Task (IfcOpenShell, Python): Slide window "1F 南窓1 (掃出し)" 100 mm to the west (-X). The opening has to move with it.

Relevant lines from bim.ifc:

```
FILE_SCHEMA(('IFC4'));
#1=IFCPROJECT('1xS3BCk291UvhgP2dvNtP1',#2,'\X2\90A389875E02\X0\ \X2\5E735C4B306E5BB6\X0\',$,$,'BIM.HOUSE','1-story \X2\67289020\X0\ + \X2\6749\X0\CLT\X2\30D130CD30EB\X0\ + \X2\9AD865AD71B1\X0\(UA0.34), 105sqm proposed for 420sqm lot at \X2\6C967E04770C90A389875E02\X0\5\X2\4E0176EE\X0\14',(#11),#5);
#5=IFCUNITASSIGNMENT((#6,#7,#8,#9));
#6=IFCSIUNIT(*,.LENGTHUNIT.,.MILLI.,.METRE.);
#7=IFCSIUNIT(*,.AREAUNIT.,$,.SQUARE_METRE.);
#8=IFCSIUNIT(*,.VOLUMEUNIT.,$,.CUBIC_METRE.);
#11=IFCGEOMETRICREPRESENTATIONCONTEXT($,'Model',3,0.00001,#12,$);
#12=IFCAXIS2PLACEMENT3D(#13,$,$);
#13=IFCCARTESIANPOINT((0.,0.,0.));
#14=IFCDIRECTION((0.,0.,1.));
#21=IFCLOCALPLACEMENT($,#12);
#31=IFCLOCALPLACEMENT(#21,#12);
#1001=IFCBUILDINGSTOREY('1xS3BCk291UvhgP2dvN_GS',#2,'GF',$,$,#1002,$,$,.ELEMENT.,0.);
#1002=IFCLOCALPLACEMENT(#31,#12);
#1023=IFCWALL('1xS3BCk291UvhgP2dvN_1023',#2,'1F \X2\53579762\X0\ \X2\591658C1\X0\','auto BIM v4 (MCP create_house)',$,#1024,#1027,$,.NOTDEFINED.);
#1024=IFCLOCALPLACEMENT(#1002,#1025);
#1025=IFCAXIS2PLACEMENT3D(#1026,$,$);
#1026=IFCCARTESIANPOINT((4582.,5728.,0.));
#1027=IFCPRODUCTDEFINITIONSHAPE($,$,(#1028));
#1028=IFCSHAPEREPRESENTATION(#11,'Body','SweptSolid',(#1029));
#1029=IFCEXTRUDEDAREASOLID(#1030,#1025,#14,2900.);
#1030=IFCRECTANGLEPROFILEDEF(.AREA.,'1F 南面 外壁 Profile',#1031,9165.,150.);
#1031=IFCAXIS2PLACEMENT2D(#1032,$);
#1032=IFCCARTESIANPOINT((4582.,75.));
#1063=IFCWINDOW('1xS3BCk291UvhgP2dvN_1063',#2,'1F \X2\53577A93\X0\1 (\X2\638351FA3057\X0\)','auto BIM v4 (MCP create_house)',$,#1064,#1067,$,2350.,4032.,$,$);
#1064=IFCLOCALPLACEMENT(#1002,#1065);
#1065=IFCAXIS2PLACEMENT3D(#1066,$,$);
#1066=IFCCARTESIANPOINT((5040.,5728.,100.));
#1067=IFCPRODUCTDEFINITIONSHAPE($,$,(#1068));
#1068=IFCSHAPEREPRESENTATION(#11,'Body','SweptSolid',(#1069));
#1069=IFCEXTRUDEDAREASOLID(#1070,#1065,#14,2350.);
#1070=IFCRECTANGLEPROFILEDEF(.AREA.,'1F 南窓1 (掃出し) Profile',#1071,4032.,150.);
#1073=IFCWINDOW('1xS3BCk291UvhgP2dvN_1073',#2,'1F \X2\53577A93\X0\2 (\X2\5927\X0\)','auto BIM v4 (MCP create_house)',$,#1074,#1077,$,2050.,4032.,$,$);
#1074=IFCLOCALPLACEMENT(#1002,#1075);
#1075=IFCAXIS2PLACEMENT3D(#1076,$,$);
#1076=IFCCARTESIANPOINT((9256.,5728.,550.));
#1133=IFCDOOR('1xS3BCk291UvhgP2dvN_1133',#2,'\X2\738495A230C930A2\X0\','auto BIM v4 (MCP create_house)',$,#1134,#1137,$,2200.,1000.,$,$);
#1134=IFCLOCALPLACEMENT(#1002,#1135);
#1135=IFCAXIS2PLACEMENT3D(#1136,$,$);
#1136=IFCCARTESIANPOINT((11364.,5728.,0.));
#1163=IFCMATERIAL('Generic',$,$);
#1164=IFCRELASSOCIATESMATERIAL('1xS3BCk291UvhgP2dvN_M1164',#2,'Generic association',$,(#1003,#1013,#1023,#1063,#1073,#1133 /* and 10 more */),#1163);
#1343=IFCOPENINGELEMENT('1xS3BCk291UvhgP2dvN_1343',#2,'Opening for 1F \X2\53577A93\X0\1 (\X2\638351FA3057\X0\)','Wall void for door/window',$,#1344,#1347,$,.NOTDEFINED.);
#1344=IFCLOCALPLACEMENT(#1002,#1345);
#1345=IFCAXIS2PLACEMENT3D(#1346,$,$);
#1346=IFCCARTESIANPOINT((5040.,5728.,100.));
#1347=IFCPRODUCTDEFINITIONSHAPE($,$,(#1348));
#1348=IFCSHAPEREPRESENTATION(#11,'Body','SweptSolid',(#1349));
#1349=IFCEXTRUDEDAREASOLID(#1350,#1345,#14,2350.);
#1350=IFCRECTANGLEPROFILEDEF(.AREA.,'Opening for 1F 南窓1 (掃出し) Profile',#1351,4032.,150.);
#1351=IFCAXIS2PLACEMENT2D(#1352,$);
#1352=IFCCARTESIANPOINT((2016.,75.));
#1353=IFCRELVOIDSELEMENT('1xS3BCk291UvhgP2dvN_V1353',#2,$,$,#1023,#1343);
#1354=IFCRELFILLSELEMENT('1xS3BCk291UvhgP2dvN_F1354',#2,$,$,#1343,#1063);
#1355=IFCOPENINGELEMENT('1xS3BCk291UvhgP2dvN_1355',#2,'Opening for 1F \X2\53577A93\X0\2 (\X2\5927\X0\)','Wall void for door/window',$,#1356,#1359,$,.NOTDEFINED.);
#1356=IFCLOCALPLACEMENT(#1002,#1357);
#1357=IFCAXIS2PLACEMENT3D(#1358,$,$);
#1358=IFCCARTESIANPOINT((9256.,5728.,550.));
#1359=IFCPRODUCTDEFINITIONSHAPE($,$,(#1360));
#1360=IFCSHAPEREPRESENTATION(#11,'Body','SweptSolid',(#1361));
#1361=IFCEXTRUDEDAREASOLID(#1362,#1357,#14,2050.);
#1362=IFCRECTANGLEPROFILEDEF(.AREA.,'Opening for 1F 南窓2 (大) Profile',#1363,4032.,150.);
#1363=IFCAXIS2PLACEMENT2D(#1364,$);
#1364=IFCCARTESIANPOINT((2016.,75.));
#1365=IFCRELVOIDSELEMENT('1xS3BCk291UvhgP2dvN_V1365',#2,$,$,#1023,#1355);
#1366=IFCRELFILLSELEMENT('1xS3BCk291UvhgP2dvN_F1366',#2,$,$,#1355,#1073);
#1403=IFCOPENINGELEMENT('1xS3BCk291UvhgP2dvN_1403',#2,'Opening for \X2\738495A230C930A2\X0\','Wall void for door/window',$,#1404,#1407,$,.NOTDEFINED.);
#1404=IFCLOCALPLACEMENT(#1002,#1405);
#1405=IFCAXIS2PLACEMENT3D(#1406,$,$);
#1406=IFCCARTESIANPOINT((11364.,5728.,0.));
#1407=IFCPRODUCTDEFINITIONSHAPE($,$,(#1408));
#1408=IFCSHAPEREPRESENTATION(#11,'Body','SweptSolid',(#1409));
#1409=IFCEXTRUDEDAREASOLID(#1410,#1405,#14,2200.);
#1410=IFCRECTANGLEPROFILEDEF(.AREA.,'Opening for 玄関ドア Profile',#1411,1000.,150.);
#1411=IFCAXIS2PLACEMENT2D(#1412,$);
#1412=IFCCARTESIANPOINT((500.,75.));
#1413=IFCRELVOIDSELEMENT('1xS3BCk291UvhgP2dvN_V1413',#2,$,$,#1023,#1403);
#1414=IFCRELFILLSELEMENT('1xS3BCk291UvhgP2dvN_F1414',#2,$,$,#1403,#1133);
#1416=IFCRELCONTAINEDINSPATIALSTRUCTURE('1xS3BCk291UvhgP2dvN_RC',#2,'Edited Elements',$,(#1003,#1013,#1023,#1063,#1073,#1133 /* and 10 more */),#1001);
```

```python
import ifcopenshell
import ifcopenshell.api.geometry
import ifcopenshell.util.placement

model = ifcopenshell.open("bim.ifc")

window = model.by_guid("1xS3BCk291UvhgP2dvN_1063")
opening = window.FillsVoids[0].RelatingOpeningElement
wall = opening.VoidsElements[0].RelatingBuildingElement

wall_matrix = ifcopenshell.util.placement.get_local_placement(wall.ObjectPlacement)
shift = wall_matrix[:3, 0] * -100.0
before = ifcopenshell.util.placement.get_local_placement(window.ObjectPlacement)[:3, 3].copy()

# The window is not placed relative to its opening, so move both.
for product in (opening, window):
    matrix = ifcopenshell.util.placement.get_local_placement(product.ObjectPlacement)
    matrix[:3, 3] += shift
    ifcopenshell.api.geometry.edit_object_placement(model, product=product, matrix=matrix, is_si=False)

after = ifcopenshell.util.placement.get_local_placement(window.ObjectPlacement)[:3, 3]
print("window moved by", (after - before).round(3) + 0.0)

model.write("bim_updated.ifc")
```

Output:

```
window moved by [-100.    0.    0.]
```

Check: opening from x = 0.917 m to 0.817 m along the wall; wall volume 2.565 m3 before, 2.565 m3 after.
